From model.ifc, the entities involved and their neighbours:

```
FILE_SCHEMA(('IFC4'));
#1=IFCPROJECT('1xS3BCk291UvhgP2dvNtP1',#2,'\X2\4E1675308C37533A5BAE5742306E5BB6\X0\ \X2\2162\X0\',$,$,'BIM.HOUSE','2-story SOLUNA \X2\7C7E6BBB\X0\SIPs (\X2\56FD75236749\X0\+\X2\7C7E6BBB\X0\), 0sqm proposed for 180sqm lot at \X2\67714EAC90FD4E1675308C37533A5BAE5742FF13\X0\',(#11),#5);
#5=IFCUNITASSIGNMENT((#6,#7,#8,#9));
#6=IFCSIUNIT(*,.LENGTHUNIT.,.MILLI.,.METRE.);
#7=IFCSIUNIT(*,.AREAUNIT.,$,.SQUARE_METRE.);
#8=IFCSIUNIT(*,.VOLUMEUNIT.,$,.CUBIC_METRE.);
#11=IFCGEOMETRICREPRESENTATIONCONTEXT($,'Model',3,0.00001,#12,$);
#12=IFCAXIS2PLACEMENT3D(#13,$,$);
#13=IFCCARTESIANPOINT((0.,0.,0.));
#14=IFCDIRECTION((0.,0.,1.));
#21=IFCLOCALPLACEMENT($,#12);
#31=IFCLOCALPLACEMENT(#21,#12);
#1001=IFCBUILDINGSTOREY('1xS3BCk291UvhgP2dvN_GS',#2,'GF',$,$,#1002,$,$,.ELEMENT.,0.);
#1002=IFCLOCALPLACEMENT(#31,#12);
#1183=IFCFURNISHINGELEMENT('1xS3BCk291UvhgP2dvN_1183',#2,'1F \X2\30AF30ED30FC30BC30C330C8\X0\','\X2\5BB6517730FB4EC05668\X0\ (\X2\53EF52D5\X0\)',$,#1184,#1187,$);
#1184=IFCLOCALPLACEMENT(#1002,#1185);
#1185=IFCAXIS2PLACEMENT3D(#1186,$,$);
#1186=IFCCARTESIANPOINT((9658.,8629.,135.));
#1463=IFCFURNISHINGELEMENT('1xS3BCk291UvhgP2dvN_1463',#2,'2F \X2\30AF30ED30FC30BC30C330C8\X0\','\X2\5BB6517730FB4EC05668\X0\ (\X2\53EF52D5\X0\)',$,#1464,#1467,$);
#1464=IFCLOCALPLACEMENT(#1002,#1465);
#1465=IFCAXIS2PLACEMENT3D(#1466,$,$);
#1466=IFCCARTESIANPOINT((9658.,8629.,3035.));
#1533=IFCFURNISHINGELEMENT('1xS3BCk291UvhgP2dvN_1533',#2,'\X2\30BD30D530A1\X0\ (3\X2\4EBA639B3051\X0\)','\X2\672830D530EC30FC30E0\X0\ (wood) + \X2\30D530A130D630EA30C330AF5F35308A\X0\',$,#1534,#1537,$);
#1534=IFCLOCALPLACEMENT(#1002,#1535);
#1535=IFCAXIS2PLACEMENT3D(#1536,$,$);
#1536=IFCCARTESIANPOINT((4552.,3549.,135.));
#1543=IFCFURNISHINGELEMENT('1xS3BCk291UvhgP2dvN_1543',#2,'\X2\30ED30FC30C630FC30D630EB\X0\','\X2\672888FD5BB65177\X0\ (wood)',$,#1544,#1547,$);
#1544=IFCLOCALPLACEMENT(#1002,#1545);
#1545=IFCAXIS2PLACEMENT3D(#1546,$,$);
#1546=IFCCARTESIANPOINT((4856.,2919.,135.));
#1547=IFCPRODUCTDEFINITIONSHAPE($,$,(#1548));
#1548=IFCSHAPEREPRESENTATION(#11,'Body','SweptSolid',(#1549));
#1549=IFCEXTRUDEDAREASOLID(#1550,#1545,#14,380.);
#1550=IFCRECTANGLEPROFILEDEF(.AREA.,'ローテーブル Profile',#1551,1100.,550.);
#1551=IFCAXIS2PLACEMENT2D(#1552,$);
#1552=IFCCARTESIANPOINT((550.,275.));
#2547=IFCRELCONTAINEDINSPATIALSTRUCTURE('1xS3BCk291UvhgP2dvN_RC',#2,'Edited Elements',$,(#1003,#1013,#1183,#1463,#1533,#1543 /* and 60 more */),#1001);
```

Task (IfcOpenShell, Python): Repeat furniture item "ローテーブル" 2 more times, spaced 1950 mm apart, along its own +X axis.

```python
import ifcopenshell
import ifcopenshell.api.geometry
import ifcopenshell.api.root
import ifcopenshell.util.element
import ifcopenshell.util.placement

model = ifcopenshell.open("model.ifc")


def reuse_history(source, copy):
    """copy_class also copies each property set's owner history, people and application; keep the originals."""
    for rel in copy.IsDefinedBy:
        if rel.is_a("IfcRelDefinesByProperties") and (history := rel.RelatingPropertyDefinition.OwnerHistory):
            rel.RelatingPropertyDefinition.OwnerHistory = source.OwnerHistory
            ifcopenshell.util.element.remove_deep2(model, history)


source = model.by_guid("1xS3BCk291UvhgP2dvN_1543")
base = ifcopenshell.util.placement.get_local_placement(source.ObjectPlacement)
step = base[:3, 0] * 1950.0

for i in range(1, 3):
    copy = ifcopenshell.api.root.copy_class(model, product=source)
    copy.Representation = ifcopenshell.util.element.copy_deep(
        model, source.Representation, exclude=["IfcGeometricRepresentationContext", "IfcRepresentationMap"]
    )
    reuse_history(source, copy)
    matrix = base.copy()
    matrix[:3, 3] += i * step
    print("added at", matrix[:3, 3].round(3) + 0.0)
    ifcopenshell.api.geometry.edit_object_placement(model, product=copy, matrix=matrix, is_si=False)

model.write("model_edited.ifc")
```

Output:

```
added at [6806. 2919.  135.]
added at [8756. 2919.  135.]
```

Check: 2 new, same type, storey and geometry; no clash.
